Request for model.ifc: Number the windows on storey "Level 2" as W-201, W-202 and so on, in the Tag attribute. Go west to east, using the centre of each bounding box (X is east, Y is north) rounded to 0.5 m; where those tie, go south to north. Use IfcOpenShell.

First a look at what the model holds.

```python
import ifcopenshell
import ifcopenshell.util.element
import ifcopenshell.util.placement

model = ifcopenshell.open("model.ifc")
print(model.schema)
storey = next(s for s in model.by_type("IfcBuildingStorey") if s.Name == "Level 2")
windows = [e for e in ifcopenshell.util.element.get_decomposition(storey) if e.is_a("IfcWindow")]
for e in sorted(windows, key=lambda e: e.id()):
    origin = ifcopenshell.util.placement.get_local_placement(e.ObjectPlacement)[:3, 3]
    print(e.id(), e.Tag, e.Name, origin.round(2) + 0.0, sep=" | ")
```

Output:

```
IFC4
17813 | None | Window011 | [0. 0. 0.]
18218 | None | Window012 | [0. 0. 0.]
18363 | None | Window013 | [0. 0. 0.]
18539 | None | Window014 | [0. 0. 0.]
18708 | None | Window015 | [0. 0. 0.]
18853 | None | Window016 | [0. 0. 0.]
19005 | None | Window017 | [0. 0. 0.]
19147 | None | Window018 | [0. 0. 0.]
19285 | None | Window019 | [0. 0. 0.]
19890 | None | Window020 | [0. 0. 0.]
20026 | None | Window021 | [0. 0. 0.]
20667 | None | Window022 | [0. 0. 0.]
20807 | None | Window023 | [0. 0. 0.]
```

```python
import ifcopenshell
import ifcopenshell.geom
import ifcopenshell.util.element
import ifcopenshell.util.shape

model = ifcopenshell.open("model.ifc")
settings = ifcopenshell.geom.settings()
settings.set("use-world-coords", True)


def centre(element):
    shape = ifcopenshell.geom.create_shape(settings, element)
    return ifcopenshell.util.shape.get_bbox_centroid(shape.geometry)


storey = next(s for s in model.by_type("IfcBuildingStorey") if s.Name == "Level 2")
windows = [e for e in ifcopenshell.util.element.get_decomposition(storey) if e.is_a("IfcWindow")]

# Insertion points can sit at a corner or the storey origin, so sort by the geometry (in metres).
centres = {e: centre(e) for e in windows}
windows.sort(key=lambda e: (round(centres[e][0] / 0.5), centres[e][1]))

for i, e in enumerate(windows, start=1):
    number = f"W-2{i:02d}"
    e.Tag = number
    print(e.id(), number)

model.write("model_edited.ifc")
```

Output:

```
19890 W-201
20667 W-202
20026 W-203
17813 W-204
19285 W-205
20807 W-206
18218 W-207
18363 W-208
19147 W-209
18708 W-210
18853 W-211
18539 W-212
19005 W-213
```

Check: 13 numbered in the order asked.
